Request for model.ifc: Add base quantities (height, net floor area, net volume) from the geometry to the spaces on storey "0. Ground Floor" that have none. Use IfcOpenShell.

First a look at what the model holds.

```python
import ifcopenshell
import ifcopenshell.util.element
import ifcopenshell.util.unit

model = ifcopenshell.open("model.ifc")
print(model.schema)
for unit_type in ("LENGTHUNIT", "AREAUNIT", "VOLUMEUNIT"):
    print(unit_type, ifcopenshell.util.unit.calculate_unit_scale(model, unit_type))
storey = next(s for s in model.by_type("IfcBuildingStorey") if s.Name == "0. Ground Floor")
spaces = [e for e in ifcopenshell.util.element.get_decomposition(storey) if e.is_a("IfcSpace")]
for e in sorted(spaces, key=lambda e: e.id()):
    print(e.id(), e.is_a(), e.Name, list(ifcopenshell.util.element.get_psets(e, qtos_only=True)), sep=" | ")
```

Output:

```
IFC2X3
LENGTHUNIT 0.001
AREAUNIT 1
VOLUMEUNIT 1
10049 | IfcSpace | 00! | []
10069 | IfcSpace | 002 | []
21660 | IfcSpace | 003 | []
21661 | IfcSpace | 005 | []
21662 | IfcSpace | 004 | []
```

```python
import ifcopenshell
import ifcopenshell.api.pset
import ifcopenshell.geom
import ifcopenshell.util.element
import ifcopenshell.util.shape
import ifcopenshell.util.unit

model = ifcopenshell.open("model.ifc")
unit_scale = ifcopenshell.util.unit.calculate_unit_scale(model)
area_scale = ifcopenshell.util.unit.calculate_unit_scale(model, "AREAUNIT")
volume_scale = ifcopenshell.util.unit.calculate_unit_scale(model, "VOLUMEUNIT")
settings = ifcopenshell.geom.settings()

storey = next(s for s in model.by_type("IfcBuildingStorey") if s.Name == "0. Ground Floor")
spaces = [e for e in ifcopenshell.util.element.get_decomposition(storey) if e.is_a("IfcSpace")]

for e in sorted(spaces, key=lambda e: e.id()):
    if ifcopenshell.util.element.get_psets(e, qtos_only=True, should_inherit=False):
        continue
    # Geometry comes back in metres, in the element's own axes.
    shape = ifcopenshell.geom.create_shape(settings, e)
    values = {
        "Height": ifcopenshell.util.shape.get_z(shape.geometry) / unit_scale,
        "NetFloorArea": ifcopenshell.util.shape.get_footprint_area(shape.geometry) / area_scale,
        "NetVolume": ifcopenshell.util.shape.get_volume(shape.geometry) / volume_scale,
    }
    qto = ifcopenshell.api.pset.add_qto(model, product=e, name="BaseQuantities")
    ifcopenshell.api.pset.edit_qto(model, qto=qto, properties=values)
    print(e.id(), {k: round(v, 3) for k, v in values.items()})

model.write("model-out.ifc")
```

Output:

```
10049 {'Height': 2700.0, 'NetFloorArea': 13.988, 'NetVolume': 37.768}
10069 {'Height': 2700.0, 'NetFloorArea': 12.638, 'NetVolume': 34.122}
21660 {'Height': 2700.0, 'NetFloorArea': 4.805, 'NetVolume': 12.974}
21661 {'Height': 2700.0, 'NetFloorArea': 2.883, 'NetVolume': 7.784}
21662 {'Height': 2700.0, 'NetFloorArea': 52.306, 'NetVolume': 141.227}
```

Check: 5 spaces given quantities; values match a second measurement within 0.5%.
